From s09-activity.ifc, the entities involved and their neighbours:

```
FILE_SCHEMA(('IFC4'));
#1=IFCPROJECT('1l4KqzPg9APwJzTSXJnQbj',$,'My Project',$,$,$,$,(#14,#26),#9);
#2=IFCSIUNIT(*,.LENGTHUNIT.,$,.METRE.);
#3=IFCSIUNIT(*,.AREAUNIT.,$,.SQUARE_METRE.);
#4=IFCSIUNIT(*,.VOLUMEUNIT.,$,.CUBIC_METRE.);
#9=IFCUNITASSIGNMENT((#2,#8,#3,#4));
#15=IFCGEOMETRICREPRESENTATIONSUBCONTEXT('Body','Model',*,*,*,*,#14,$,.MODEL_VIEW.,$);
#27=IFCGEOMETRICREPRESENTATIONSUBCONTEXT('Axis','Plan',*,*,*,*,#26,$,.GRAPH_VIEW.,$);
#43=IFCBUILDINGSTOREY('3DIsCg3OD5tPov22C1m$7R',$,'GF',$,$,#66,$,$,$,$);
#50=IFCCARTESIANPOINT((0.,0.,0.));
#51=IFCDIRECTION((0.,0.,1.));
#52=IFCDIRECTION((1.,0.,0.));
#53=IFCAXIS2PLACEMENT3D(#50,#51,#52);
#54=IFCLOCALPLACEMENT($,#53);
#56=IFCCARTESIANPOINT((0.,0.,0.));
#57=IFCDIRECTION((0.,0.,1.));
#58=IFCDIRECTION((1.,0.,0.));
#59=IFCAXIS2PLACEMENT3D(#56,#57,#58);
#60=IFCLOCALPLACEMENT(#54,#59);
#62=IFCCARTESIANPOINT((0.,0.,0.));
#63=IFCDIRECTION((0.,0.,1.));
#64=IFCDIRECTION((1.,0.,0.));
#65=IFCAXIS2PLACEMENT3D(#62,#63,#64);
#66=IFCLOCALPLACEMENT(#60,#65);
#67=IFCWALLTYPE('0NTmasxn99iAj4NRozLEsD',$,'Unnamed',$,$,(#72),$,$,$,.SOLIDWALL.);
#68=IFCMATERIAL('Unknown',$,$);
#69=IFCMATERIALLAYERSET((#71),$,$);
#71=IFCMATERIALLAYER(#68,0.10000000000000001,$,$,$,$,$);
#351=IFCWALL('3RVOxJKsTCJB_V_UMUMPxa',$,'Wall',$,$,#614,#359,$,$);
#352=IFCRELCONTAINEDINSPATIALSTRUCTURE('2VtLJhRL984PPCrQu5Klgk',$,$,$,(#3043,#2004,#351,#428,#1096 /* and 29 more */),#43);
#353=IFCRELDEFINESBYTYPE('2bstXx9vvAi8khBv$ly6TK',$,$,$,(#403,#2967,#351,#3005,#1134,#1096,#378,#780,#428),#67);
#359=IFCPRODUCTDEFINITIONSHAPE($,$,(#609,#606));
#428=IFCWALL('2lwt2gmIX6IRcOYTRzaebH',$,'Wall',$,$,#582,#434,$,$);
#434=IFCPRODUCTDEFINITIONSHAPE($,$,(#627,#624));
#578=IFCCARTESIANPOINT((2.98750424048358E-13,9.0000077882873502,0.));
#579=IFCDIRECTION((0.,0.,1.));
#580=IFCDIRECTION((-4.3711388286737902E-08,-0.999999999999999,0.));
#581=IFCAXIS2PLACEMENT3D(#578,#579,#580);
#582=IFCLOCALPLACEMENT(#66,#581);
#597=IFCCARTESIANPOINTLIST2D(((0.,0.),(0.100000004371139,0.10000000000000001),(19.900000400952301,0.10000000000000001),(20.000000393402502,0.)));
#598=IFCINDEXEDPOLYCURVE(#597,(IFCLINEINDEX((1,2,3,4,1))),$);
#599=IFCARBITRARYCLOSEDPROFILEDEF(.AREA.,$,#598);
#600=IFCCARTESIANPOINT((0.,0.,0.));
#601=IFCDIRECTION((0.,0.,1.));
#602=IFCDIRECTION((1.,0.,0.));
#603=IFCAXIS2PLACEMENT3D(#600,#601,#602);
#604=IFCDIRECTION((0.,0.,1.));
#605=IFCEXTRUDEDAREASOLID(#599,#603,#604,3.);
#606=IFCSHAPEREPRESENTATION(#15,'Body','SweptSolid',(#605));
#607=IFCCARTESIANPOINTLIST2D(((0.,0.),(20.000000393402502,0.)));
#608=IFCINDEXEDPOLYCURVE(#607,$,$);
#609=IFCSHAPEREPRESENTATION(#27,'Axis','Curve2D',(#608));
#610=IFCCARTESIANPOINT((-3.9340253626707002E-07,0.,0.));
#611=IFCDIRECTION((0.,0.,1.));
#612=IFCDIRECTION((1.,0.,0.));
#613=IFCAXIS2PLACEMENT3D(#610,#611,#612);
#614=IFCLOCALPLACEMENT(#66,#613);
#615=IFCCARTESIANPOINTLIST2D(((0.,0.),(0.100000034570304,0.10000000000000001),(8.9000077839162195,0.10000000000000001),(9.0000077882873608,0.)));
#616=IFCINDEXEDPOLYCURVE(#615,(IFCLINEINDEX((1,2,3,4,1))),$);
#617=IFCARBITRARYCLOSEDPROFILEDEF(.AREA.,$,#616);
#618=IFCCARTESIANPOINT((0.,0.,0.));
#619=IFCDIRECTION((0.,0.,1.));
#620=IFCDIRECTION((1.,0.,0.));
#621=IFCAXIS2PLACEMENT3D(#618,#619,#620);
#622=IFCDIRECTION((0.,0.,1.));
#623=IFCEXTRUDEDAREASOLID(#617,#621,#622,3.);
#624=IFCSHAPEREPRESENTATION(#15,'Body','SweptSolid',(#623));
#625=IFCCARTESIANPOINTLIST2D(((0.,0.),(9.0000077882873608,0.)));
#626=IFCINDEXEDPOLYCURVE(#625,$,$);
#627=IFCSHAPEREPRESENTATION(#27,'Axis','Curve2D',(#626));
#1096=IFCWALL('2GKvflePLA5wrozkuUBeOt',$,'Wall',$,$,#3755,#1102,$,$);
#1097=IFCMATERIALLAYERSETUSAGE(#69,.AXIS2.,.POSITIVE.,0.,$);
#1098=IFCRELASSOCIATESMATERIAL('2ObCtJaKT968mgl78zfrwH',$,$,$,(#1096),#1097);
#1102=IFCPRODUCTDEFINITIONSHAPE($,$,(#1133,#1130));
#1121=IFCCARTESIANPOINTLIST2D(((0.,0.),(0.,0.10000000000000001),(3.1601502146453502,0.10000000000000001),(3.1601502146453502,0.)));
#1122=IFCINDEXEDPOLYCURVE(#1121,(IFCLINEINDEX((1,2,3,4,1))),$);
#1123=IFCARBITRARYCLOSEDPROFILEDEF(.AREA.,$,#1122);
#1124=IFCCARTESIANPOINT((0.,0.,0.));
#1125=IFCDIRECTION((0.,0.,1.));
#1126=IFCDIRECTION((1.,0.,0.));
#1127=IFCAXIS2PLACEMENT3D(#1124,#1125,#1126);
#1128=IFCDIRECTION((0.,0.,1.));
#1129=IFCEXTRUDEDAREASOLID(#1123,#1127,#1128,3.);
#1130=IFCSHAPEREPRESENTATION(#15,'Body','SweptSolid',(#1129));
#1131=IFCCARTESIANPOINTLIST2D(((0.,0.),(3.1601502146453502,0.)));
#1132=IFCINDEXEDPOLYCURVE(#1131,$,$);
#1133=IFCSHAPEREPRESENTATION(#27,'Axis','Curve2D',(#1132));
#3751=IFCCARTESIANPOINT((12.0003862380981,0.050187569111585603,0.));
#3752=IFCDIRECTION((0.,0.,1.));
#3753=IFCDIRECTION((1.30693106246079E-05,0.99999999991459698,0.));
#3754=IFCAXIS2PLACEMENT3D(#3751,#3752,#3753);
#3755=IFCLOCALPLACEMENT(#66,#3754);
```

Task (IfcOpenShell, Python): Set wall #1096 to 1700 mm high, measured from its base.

```python
import ifcopenshell
import ifcopenshell.geom
import ifcopenshell.util.representation
import ifcopenshell.util.shape
import ifcopenshell.util.unit

model = ifcopenshell.open("s09-activity.ifc")
unit_scale = ifcopenshell.util.unit.calculate_unit_scale(model)
settings = ifcopenshell.geom.settings()


def volume(element):
    """Net volume in cubic metres, openings subtracted."""
    shape = ifcopenshell.geom.create_shape(settings, element)
    return ifcopenshell.util.shape.get_volume(shape.geometry)


wall = model.by_id(1096)
before = volume(wall)

body = ifcopenshell.util.representation.get_representation(wall, "Model", "Body")
solid = body.Items[0]
old_height = solid.Depth
solid.Depth = 1.7 / unit_scale
after = volume(wall)

print(f"height {old_height:g} -> {solid.Depth:g}, volume {before:.3f} -> {after:.3f} m3")

model.write("s09-activity_edited.ifc")
```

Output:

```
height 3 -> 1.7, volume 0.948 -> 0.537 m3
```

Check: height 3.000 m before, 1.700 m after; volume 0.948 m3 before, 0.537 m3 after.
